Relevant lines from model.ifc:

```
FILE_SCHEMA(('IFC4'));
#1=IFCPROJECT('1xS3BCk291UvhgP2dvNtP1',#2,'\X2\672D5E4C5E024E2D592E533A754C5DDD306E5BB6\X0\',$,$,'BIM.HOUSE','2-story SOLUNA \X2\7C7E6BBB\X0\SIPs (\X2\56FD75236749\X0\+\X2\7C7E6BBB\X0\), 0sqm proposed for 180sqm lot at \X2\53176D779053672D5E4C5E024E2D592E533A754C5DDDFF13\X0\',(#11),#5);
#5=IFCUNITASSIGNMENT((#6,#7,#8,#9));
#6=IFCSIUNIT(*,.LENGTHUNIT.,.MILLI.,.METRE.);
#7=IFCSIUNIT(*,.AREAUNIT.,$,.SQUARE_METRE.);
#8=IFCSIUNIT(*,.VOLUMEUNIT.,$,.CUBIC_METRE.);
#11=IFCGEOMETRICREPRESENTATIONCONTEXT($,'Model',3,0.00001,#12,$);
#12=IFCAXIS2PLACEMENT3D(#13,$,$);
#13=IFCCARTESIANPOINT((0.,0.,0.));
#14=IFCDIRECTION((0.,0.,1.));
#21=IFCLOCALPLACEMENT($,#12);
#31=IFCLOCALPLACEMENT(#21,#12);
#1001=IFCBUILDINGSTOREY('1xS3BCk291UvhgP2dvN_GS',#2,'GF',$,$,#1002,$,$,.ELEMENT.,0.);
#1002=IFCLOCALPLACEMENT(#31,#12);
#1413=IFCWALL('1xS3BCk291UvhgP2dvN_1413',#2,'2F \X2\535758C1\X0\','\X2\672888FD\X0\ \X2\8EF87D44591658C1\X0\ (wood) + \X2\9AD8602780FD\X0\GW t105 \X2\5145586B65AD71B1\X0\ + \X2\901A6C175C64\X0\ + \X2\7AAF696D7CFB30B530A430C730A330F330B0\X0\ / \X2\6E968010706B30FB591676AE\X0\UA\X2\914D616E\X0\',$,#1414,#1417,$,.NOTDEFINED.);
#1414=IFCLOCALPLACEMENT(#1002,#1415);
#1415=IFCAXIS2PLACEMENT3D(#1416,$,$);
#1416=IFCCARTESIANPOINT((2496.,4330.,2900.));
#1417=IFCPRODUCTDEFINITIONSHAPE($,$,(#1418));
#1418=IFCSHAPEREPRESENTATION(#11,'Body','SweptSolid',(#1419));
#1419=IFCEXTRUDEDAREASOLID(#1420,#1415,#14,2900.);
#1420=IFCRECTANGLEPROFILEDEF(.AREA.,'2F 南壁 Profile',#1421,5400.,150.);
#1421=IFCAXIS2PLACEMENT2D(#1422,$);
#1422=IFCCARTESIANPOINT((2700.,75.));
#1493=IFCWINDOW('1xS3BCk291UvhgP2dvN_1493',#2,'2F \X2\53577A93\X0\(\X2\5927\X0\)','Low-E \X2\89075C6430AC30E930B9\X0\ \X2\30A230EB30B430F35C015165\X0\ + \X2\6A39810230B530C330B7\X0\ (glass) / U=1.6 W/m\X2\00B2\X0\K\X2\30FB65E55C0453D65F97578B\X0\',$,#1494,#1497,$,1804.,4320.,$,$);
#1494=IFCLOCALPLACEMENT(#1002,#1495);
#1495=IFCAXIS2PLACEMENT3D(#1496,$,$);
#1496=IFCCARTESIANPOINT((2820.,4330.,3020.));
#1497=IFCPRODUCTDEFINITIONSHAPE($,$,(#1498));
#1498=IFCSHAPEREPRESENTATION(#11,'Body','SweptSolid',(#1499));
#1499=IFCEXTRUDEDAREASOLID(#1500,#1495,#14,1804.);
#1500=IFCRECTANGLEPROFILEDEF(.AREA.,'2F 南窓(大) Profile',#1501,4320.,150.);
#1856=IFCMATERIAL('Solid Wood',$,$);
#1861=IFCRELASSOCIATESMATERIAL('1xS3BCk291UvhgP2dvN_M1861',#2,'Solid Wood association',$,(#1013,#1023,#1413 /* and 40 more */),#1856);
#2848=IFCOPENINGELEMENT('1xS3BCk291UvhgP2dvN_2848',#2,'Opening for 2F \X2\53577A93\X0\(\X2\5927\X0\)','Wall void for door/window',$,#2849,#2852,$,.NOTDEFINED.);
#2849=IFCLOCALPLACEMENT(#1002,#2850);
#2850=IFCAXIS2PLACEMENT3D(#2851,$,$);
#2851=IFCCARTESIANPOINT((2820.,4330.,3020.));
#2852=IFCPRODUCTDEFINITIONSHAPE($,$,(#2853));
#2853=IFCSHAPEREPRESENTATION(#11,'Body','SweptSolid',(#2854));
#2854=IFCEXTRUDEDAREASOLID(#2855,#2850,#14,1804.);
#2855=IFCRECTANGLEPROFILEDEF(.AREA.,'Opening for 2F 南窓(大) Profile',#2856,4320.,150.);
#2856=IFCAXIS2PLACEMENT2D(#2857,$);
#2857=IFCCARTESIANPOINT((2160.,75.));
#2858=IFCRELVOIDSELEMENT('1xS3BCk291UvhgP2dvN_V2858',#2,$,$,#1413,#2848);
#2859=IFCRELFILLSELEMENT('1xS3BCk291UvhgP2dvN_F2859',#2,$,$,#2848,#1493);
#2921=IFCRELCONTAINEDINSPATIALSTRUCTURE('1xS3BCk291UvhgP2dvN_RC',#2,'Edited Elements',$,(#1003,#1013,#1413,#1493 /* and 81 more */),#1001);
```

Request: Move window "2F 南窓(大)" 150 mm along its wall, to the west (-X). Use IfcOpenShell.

```python
import ifcopenshell
import ifcopenshell.api.geometry
import ifcopenshell.util.placement
import ifcopenshell.util.unit

model = ifcopenshell.open("model.ifc")
unit_scale = ifcopenshell.util.unit.calculate_unit_scale(model)

window = model.by_id(1493)
opening = window.FillsVoids[0].RelatingOpeningElement
wall = opening.VoidsElements[0].RelatingBuildingElement

wall_matrix = ifcopenshell.util.placement.get_local_placement(wall.ObjectPlacement)
shift = wall_matrix[:3, 0] * -0.15 / unit_scale
before = ifcopenshell.util.placement.get_local_placement(window.ObjectPlacement)[:3, 3].copy()

# The window is not placed relative to its opening, so move both.
for product in (opening, window):
    matrix = ifcopenshell.util.placement.get_local_placement(product.ObjectPlacement)
    matrix[:3, 3] += shift
    ifcopenshell.api.geometry.edit_object_placement(model, product=product, matrix=matrix, is_si=False)

after = ifcopenshell.util.placement.get_local_placement(window.ObjectPlacement)[:3, 3]
print("window moved by", (after - before).round(3) + 0.0)

model.write("model_rev.ifc")
```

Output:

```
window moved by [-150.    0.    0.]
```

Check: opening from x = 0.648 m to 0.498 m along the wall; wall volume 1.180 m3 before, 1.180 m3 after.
